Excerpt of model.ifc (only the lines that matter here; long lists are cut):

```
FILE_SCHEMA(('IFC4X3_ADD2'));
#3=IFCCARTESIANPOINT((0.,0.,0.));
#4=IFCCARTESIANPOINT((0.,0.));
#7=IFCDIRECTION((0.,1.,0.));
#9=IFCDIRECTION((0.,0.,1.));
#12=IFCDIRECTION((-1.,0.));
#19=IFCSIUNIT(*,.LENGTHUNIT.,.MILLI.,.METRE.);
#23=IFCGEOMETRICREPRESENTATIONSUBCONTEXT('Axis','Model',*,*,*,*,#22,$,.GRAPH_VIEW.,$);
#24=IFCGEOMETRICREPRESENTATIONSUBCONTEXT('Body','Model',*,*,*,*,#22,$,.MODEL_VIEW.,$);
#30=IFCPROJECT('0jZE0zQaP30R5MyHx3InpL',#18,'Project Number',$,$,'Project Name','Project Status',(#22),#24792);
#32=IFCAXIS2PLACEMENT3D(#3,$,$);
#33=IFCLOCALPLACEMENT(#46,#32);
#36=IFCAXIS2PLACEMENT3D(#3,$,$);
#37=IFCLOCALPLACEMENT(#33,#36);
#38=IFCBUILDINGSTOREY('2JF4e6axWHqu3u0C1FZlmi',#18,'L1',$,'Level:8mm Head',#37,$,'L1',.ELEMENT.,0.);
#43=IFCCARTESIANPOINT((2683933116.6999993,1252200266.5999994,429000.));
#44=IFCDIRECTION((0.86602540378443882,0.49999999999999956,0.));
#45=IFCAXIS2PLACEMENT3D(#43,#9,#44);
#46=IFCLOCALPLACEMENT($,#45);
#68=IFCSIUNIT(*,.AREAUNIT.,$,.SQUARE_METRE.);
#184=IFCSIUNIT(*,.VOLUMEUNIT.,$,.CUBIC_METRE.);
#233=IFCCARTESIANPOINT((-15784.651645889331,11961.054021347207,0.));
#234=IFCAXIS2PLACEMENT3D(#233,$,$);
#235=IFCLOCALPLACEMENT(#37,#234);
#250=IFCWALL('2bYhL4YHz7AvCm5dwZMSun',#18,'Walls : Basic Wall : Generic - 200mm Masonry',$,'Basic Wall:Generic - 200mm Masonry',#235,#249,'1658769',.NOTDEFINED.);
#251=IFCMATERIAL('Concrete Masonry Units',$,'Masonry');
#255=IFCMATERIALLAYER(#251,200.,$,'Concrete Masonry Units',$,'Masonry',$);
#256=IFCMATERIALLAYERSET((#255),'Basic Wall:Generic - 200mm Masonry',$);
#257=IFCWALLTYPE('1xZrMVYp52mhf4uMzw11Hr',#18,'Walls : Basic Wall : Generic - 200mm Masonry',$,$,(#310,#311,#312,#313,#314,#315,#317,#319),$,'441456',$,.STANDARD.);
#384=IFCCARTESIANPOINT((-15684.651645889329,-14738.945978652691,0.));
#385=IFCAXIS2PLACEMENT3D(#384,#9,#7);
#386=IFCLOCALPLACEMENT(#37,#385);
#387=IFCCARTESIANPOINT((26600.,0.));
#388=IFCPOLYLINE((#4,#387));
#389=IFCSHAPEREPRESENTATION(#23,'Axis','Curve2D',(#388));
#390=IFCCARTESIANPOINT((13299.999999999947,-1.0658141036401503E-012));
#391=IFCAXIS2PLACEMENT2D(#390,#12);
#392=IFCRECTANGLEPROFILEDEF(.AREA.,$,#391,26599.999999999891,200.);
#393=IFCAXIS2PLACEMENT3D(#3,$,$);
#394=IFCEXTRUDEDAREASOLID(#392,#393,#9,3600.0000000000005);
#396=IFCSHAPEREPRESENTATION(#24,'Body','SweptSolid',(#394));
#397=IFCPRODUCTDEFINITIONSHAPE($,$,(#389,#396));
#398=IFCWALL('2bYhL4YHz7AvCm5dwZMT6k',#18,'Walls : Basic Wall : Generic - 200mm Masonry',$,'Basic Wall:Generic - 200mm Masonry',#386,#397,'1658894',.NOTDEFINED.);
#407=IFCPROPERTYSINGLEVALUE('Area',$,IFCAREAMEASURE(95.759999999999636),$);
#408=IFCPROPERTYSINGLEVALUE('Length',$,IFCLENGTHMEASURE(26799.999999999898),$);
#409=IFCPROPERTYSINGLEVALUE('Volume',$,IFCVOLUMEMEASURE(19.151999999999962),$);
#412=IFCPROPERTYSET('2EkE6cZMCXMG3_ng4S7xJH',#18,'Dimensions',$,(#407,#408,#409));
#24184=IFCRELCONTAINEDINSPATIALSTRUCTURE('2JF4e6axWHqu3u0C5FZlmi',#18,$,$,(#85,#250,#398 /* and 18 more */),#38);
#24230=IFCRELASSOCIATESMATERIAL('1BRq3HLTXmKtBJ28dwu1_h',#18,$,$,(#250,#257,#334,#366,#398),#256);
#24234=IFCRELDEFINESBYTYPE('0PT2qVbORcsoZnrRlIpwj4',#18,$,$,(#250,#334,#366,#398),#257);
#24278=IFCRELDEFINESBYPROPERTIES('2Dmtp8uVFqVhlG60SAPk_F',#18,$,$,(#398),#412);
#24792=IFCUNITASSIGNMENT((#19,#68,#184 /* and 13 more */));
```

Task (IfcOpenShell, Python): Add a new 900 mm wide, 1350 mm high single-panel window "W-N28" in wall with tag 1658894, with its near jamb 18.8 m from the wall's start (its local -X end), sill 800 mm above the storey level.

```python
import numpy as np
import ifcopenshell
import ifcopenshell.api.feature
import ifcopenshell.api.geometry
import ifcopenshell.api.pset
import ifcopenshell.api.root
import ifcopenshell.api.spatial
import ifcopenshell.geom
import ifcopenshell.util.element
import ifcopenshell.util.placement
import ifcopenshell.util.representation
import ifcopenshell.util.shape
import ifcopenshell.util.unit

model = ifcopenshell.open("model.ifc")
unit_scale = ifcopenshell.util.unit.calculate_unit_scale(model)
area_scale = ifcopenshell.util.unit.calculate_unit_scale(model, "AREAUNIT")
volume_scale = ifcopenshell.util.unit.calculate_unit_scale(model, "VOLUMEUNIT")
settings = ifcopenshell.geom.settings()


def volume(element):
    """Net volume in cubic metres, openings subtracted."""
    shape = ifcopenshell.geom.create_shape(settings, element)
    return ifcopenshell.util.shape.get_volume(shape.geometry)


wall = model.by_guid("2bYhL4YHz7AvCm5dwZMT6k")
storey = ifcopenshell.util.element.get_container(wall, ifc_class="IfcBuildingStorey")
context = ifcopenshell.util.representation.get_context(model, "Model", "Body", "MODEL_VIEW")
before = volume(wall)

width, height, from_end, sill = 0.9, 1.35, 18.8, 0.8  # metres

# The wall runs along its own X axis, and the end named is its -X end.
wall_shape = ifcopenshell.geom.create_shape(settings, wall)
x, y, z = ifcopenshell.util.shape.get_vertices(wall_shape.geometry).T
start = x.min() + from_end
face, thickness = float(y.min()), float(y.max() - y.min())
wall_matrix = ifcopenshell.util.placement.get_local_placement(wall.ObjectPlacement)
level = ifcopenshell.util.placement.get_local_placement(storey.ObjectPlacement)[2, 3]


def in_wall(x, y):
    """Placement at x, y metres in the wall's axes, at sill height."""
    matrix = wall_matrix.copy()
    matrix[:, 3] = wall_matrix @ np.array([x / unit_scale, y / unit_scale, 0.0, 1.0])
    matrix[2, 3] = level + sill / unit_scale
    return matrix


# Opening: a box that overshoots both wall faces by 50 mm.
opening = ifcopenshell.api.root.create_entity(model, ifc_class="IfcOpeningElement", predefined_type="OPENING")
box = ifcopenshell.api.geometry.add_wall_representation(
    model, context=context, length=width, height=height, thickness=thickness + 0.1
)
ifcopenshell.api.geometry.assign_representation(model, product=opening, representation=box)
ifcopenshell.api.geometry.edit_object_placement(model, product=opening, matrix=in_wall(start, face - 0.05), is_si=False)
ifcopenshell.api.feature.add_feature(model, feature=opening, element=wall)

window = ifcopenshell.api.root.create_entity(model, ifc_class="IfcWindow", name="W-N28", predefined_type="WINDOW")
window.OverallWidth, window.OverallHeight = width / unit_scale, height / unit_scale
window.PartitioningType = "SINGLE_PANEL"
body = ifcopenshell.api.geometry.add_window_representation(
    model,
    context=context,
    overall_width=window.OverallWidth,
    overall_height=window.OverallHeight,
    partition_type="SINGLE_PANEL",
)
ifcopenshell.api.geometry.assign_representation(model, product=window, representation=body)
ifcopenshell.api.spatial.assign_container(model, products=[window], relating_structure=storey)
ifcopenshell.api.feature.add_filling(model, opening=opening, element=window)

# Centre the window in the wall's thickness.
ifcopenshell.api.geometry.edit_object_placement(model, product=window, matrix=in_wall(start, face), is_si=False)
window_shape = ifcopenshell.geom.create_shape(settings, window)
depth = ifcopenshell.util.shape.get_vertices(window_shape.geometry)[:, 1]
offset = face + thickness / 2 - (depth.min() + depth.max()) / 2
ifcopenshell.api.geometry.edit_object_placement(model, product=window, matrix=in_wall(start, offset), is_si=False)

after = volume(wall)

# Update the wall's stored quantities.
pset = model.by_id(ifcopenshell.util.element.get_pset(wall, "Dimensions", should_inherit=False)["id"])
ifcopenshell.api.pset.edit_pset(model, pset=pset, properties={
    "Area": model.create_entity("IfcAreaMeasure", after / thickness / area_scale),
    "Volume": model.create_entity("IfcVolumeMeasure", after / volume_scale),
})

print(f"wall volume {before:.3f} -> {after:.3f} m3")

model.write("model_updated.ifc")
```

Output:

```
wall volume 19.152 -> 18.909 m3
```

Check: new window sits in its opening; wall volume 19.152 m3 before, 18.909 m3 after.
